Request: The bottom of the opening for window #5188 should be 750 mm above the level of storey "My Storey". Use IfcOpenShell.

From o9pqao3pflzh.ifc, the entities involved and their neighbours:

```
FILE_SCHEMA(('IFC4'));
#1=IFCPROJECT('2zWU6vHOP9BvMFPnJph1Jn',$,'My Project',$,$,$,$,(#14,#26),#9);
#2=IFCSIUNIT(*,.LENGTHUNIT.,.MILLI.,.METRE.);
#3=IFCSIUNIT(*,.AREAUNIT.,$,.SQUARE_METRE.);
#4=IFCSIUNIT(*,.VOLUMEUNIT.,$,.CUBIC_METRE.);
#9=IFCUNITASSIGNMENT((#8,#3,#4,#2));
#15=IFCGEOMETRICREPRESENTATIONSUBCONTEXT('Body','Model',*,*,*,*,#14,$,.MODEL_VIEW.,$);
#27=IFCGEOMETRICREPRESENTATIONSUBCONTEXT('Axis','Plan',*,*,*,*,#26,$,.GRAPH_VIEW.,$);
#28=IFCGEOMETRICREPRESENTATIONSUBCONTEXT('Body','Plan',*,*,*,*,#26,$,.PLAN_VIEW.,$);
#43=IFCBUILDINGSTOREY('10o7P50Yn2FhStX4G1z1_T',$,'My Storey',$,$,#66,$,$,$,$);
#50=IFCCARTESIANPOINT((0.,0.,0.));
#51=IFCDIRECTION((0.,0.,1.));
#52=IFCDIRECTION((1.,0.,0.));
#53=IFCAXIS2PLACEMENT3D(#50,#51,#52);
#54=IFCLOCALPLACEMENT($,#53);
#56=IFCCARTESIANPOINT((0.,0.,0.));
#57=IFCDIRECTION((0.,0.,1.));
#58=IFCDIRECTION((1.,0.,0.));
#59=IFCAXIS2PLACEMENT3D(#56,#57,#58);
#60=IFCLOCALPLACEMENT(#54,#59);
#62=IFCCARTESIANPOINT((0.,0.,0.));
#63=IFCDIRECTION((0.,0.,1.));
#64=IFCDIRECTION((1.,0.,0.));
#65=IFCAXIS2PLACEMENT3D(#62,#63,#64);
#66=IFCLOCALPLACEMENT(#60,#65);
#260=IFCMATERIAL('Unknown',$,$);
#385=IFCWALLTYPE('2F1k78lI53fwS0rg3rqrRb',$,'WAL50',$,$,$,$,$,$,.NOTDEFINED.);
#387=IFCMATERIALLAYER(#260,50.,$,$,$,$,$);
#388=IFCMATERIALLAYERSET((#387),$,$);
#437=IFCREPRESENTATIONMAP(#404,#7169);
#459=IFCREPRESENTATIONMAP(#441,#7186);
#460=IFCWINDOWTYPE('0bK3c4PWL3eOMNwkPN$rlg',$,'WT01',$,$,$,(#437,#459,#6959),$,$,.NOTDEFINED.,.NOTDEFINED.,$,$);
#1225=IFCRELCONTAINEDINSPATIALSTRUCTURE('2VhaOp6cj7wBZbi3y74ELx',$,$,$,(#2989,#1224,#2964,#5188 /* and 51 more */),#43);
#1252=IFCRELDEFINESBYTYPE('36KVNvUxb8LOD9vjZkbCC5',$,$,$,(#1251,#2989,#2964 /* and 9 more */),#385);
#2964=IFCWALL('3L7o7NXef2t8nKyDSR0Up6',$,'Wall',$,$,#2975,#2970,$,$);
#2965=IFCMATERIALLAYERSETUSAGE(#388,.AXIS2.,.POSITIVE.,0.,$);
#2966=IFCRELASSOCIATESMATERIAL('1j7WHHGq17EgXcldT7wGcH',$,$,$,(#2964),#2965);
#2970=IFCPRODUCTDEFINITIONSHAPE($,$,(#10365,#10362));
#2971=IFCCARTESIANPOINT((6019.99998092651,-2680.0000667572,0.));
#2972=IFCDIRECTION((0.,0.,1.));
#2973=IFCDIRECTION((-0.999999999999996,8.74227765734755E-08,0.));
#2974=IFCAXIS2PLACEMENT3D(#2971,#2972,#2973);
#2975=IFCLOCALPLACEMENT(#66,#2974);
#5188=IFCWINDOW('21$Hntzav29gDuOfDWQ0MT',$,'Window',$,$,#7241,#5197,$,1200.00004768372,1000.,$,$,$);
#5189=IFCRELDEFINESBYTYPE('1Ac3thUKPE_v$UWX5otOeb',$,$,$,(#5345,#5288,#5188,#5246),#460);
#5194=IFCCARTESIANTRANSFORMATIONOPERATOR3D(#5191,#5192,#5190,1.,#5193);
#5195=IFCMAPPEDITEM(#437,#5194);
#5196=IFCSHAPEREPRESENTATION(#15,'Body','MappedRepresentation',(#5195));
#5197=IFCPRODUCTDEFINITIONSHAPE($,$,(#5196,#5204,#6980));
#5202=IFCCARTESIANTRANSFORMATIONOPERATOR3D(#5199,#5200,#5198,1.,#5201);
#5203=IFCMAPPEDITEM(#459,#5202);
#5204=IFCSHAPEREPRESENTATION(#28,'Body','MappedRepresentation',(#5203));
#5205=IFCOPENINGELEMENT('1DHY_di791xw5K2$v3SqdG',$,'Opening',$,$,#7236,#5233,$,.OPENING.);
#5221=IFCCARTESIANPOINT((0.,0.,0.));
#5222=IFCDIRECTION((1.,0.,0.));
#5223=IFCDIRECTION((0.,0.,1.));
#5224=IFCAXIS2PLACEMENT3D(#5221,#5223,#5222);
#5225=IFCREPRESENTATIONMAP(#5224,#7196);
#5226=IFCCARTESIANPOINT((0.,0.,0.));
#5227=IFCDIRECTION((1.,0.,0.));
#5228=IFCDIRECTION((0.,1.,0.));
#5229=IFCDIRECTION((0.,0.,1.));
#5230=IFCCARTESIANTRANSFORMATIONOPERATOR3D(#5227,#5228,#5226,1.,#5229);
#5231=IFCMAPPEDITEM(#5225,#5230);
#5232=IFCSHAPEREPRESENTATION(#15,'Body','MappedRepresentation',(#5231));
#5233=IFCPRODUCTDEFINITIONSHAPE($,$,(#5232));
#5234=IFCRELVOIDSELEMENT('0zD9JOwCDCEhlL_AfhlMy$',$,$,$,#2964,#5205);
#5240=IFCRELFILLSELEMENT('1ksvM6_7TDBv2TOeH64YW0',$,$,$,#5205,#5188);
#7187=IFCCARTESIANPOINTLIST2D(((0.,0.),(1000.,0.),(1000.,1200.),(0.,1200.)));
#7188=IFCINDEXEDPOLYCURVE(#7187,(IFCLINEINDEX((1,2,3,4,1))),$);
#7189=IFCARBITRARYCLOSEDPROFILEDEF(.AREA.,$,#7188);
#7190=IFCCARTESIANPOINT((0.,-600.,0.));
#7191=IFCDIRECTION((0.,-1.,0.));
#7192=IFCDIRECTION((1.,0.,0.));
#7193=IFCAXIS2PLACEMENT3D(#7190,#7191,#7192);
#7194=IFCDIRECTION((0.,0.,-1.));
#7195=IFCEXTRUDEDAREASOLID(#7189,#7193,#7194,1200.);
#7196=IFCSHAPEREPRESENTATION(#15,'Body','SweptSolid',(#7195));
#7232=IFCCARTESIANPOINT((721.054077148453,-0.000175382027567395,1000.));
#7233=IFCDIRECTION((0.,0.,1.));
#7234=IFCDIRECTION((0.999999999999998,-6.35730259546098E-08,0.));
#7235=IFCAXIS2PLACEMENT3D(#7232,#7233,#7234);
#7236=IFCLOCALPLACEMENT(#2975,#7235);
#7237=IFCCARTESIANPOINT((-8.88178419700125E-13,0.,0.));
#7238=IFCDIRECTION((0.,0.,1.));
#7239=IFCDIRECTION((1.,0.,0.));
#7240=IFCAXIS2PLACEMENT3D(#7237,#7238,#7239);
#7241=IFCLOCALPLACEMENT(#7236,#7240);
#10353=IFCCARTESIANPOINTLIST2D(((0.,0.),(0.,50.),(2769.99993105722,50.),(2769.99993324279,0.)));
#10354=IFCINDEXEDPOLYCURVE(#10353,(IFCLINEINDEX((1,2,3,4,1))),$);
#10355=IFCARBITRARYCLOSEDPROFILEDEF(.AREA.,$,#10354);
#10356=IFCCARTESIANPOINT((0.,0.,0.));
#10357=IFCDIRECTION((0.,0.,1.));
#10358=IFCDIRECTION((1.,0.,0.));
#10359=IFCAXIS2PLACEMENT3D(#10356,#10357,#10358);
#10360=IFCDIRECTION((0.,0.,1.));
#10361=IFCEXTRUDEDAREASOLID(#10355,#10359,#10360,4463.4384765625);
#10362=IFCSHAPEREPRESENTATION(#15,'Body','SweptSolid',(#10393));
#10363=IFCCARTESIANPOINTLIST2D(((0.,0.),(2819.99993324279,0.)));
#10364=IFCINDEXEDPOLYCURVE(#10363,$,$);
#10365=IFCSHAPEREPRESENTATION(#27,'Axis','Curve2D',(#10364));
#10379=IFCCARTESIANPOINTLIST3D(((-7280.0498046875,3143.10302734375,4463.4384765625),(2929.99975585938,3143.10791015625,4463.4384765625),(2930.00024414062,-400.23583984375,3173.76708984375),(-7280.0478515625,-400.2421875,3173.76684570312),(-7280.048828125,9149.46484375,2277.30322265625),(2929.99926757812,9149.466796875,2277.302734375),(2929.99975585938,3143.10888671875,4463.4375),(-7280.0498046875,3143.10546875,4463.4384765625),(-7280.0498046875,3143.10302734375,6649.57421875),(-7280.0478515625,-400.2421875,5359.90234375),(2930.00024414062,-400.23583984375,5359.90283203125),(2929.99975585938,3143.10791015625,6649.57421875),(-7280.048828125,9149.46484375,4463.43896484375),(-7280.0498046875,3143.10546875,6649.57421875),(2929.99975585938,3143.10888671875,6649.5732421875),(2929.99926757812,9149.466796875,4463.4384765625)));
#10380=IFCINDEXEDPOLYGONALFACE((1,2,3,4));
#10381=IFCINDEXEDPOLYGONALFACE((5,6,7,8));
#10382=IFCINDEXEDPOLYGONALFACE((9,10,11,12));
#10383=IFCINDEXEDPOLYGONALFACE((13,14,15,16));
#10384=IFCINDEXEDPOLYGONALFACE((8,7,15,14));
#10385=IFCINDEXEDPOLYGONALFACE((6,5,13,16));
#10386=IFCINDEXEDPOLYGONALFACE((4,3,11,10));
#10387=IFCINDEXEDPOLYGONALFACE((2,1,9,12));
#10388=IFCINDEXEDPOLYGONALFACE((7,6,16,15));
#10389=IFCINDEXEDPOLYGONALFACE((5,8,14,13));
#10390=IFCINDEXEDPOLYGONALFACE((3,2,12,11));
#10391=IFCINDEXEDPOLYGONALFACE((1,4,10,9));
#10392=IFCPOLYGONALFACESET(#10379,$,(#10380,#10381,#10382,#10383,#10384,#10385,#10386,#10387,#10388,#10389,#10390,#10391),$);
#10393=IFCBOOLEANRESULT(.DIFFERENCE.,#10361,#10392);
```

```python
import numpy as np
import ifcopenshell
import ifcopenshell.api.geometry
import ifcopenshell.geom
import ifcopenshell.util.element
import ifcopenshell.util.placement
import ifcopenshell.util.shape
import ifcopenshell.util.unit

model = ifcopenshell.open("o9pqao3pflzh.ifc")
unit_scale = ifcopenshell.util.unit.calculate_unit_scale(model)

window = model.by_id(5188)
opening = window.FillsVoids[0].RelatingOpeningElement
storey = ifcopenshell.util.element.get_container(window, ifc_class="IfcBuildingStorey")
level = ifcopenshell.util.placement.get_local_placement(storey.ObjectPlacement)[2, 3]

# The opening's origin need not be at the sill, so measure its lowest point.
shape = ifcopenshell.geom.create_shape(ifcopenshell.geom.settings(), opening)
bottom = ifcopenshell.util.shape.get_shape_bottom_elevation(shape, shape.geometry) / unit_scale
dz = level + 0.75 / unit_scale - bottom

shift = np.array([0.0, 0.0, dz])
# The window is placed relative to its opening, so it follows when the opening moves.
matrix = ifcopenshell.util.placement.get_local_placement(opening.ObjectPlacement)
matrix[:3, 3] += shift
ifcopenshell.api.geometry.edit_object_placement(
    model, product=opening, matrix=matrix, is_si=False, should_transform_children=True
)

print(f"moved by {dz * unit_scale:+.3f} m")

model.write("o9pqao3pflzh_rev.ifc")
```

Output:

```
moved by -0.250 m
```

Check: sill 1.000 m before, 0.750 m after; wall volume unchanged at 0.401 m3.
